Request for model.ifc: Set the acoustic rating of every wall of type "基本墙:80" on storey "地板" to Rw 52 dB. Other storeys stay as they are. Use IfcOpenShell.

First a look at what the model holds.

```python
import ifcopenshell
import ifcopenshell.util.element

model = ifcopenshell.open("model.ifc")
print(model.schema)
storey = next(s for s in model.by_type("IfcBuildingStorey") if s.Name == "地板")
walls = [e for e in ifcopenshell.util.element.get_decomposition(storey) if e.is_a("IfcWall")]
seen = {}
for e in walls:
    element_type = ifcopenshell.util.element.get_type(e)
    key = (element_type.Name if element_type != e and element_type else None, ifcopenshell.util.element.get_pset(e, "Pset_WallCommon", "AcousticRating"))
    seen[key] = seen.get(key, 0) + 1
for (name, value), count in sorted(seen.items(), key=str):
    print(count, "x", name, "|", value)
```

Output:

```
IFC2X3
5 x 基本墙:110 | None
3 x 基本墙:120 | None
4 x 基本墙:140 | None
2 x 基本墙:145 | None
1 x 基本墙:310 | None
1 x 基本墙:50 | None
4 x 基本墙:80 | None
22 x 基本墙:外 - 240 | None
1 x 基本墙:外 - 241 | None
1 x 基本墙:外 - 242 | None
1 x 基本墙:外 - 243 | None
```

```python
import ifcopenshell
import ifcopenshell.api.pset
import ifcopenshell.util.element

model = ifcopenshell.open("model.ifc")

storey = next(s for s in model.by_type("IfcBuildingStorey") if s.Name == "地板")
walls = [e for e in ifcopenshell.util.element.get_decomposition(storey) if e.is_a("IfcWall")]

count = 0
for e in walls:
    element_type = ifcopenshell.util.element.get_type(e)
    if element_type in (None, e) or element_type.Name != "基本墙:80":
        continue
    # add_pset returns the element's existing set when there is one.
    pset = ifcopenshell.api.pset.add_pset(model, product=e, name="Pset_WallCommon")
    ifcopenshell.api.pset.edit_pset(model, pset=pset, properties={"AcousticRating": "Rw 52 dB"})
    count += 1

print(count, "walls updated")

model.write("model-out.ifc")
```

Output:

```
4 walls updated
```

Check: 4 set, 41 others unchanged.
